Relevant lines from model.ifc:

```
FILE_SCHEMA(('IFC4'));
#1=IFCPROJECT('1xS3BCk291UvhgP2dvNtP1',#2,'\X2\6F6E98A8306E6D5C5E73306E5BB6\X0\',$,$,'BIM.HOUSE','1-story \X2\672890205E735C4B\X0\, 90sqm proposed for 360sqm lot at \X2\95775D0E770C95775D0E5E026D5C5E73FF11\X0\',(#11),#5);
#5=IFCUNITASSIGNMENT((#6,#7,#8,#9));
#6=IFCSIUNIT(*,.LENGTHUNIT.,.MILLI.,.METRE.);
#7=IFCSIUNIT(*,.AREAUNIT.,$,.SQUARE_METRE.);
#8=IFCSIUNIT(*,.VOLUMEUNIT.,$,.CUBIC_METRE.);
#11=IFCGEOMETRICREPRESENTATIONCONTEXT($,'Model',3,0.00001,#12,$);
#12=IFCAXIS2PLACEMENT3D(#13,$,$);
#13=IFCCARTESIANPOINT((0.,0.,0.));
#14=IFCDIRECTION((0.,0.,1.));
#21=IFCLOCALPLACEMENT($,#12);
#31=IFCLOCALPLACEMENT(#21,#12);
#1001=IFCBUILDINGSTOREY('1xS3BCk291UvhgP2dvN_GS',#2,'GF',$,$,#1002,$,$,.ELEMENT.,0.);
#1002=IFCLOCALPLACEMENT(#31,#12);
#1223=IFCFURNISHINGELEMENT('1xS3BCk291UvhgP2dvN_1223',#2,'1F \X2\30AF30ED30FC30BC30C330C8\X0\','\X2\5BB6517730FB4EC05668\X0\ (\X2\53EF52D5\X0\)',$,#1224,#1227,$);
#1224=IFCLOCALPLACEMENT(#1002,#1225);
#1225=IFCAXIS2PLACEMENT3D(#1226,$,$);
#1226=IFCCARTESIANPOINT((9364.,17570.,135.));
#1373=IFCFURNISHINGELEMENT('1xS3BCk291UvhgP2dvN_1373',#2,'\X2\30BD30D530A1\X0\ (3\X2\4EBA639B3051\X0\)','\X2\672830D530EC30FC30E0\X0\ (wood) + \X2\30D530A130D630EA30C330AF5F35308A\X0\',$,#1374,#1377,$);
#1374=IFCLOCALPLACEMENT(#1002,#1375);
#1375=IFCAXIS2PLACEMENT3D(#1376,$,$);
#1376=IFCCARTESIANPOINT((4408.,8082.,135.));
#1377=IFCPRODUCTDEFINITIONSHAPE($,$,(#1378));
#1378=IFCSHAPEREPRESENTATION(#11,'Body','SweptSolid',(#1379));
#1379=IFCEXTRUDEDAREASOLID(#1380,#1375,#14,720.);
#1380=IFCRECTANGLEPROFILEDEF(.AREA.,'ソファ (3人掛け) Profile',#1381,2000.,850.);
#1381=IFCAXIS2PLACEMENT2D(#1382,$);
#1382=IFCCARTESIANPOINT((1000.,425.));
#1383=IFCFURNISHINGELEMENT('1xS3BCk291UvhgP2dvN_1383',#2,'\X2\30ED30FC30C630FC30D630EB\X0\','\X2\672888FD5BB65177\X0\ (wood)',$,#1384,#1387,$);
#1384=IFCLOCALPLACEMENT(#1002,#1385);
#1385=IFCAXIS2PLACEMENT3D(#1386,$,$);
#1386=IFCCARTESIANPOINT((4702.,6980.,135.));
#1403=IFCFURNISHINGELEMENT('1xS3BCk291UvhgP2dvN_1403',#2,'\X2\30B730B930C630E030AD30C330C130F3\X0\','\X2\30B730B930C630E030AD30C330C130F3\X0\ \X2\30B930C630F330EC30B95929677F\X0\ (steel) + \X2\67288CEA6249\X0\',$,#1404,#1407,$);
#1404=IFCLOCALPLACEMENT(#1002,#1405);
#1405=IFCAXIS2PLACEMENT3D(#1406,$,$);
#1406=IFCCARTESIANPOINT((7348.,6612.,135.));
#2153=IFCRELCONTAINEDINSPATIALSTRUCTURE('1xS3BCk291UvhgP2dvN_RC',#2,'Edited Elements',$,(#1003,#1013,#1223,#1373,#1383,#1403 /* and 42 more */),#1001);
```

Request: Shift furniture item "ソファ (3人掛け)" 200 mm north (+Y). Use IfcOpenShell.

```python
import ifcopenshell
import ifcopenshell.api.geometry
import ifcopenshell.util.placement
import ifcopenshell.util.unit

model = ifcopenshell.open("model.ifc")
unit_scale = ifcopenshell.util.unit.calculate_unit_scale(model)

item = model.by_id(1373)
matrix = ifcopenshell.util.placement.get_local_placement(item.ObjectPlacement)
matrix[1, 3] += 0.2 / unit_scale
ifcopenshell.api.geometry.edit_object_placement(model, product=item, matrix=matrix, is_si=False)

print(ifcopenshell.util.placement.get_local_placement(item.ObjectPlacement).round(3) + 0.0)

model.write("model_edited.ifc")
```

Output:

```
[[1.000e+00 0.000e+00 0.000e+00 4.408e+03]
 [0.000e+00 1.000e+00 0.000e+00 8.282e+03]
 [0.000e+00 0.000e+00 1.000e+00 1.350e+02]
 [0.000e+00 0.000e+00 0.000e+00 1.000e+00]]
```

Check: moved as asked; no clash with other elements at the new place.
